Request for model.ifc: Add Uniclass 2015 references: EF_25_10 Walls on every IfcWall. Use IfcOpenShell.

First a look at what the model holds.

```python
import ifcopenshell

model = ifcopenshell.open("model.ifc")
print(model.schema)
print("classifications:", [c.Name for c in model.by_type("IfcClassification")])
for ifc_class in ("IfcDoor", "IfcRoof", "IfcStair", "IfcWall", "IfcWindow"):
    print(ifc_class, len(model.by_type(ifc_class)))
```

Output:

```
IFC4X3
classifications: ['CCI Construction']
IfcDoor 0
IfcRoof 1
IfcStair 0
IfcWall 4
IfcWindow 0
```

```python
import ifcopenshell
import ifcopenshell.api.classification

model = ifcopenshell.open("model.ifc")

system = ifcopenshell.api.classification.add_classification(model, classification="Uniclass 2015")

codes = {
    "IfcWall": ("EF_25_10", "Walls"),
}
for ifc_class, (code, name) in codes.items():
    products = model.by_type(ifc_class)
    ifcopenshell.api.classification.add_reference(
        model, products=products, classification=system, identification=code, name=name
    )
    print(code, len(products))

model.write("model_updated.ifc")
```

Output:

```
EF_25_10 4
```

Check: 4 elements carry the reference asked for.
